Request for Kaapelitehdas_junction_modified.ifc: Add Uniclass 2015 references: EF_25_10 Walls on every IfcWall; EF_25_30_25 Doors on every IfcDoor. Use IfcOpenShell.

First a look at what the model holds.

```python
import ifcopenshell

model = ifcopenshell.open("Kaapelitehdas_junction_modified.ifc")
print(model.schema)
print("classifications:", [c.Name for c in model.by_type("IfcClassification")])
for ifc_class in ("IfcDoor", "IfcRoof", "IfcStair", "IfcWall", "IfcWindow"):
    print(ifc_class, len(model.by_type(ifc_class)))
```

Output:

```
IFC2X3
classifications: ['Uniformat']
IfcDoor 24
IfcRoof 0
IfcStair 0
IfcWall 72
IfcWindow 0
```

```python
import ifcopenshell
import ifcopenshell.api.classification

model = ifcopenshell.open("Kaapelitehdas_junction_modified.ifc")

# IFC2X3 requires Source and Edition and has no link from the project to the system.
system = model.create_entity("IfcClassification", Source="NBS", Edition="2015", Name="Uniclass 2015")

codes = {
    "IfcWall": ("EF_25_10", "Walls"),
    "IfcDoor": ("EF_25_30_25", "Doors"),
}
for ifc_class, (code, name) in codes.items():
    products = model.by_type(ifc_class)
    ifcopenshell.api.classification.add_reference(
        model, products=products, classification=system, identification=code, name=name
    )
    print(code, len(products))

model.write("Kaapelitehdas_junction_modified_v2.ifc")
```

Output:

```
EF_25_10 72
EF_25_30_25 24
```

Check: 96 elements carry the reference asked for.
